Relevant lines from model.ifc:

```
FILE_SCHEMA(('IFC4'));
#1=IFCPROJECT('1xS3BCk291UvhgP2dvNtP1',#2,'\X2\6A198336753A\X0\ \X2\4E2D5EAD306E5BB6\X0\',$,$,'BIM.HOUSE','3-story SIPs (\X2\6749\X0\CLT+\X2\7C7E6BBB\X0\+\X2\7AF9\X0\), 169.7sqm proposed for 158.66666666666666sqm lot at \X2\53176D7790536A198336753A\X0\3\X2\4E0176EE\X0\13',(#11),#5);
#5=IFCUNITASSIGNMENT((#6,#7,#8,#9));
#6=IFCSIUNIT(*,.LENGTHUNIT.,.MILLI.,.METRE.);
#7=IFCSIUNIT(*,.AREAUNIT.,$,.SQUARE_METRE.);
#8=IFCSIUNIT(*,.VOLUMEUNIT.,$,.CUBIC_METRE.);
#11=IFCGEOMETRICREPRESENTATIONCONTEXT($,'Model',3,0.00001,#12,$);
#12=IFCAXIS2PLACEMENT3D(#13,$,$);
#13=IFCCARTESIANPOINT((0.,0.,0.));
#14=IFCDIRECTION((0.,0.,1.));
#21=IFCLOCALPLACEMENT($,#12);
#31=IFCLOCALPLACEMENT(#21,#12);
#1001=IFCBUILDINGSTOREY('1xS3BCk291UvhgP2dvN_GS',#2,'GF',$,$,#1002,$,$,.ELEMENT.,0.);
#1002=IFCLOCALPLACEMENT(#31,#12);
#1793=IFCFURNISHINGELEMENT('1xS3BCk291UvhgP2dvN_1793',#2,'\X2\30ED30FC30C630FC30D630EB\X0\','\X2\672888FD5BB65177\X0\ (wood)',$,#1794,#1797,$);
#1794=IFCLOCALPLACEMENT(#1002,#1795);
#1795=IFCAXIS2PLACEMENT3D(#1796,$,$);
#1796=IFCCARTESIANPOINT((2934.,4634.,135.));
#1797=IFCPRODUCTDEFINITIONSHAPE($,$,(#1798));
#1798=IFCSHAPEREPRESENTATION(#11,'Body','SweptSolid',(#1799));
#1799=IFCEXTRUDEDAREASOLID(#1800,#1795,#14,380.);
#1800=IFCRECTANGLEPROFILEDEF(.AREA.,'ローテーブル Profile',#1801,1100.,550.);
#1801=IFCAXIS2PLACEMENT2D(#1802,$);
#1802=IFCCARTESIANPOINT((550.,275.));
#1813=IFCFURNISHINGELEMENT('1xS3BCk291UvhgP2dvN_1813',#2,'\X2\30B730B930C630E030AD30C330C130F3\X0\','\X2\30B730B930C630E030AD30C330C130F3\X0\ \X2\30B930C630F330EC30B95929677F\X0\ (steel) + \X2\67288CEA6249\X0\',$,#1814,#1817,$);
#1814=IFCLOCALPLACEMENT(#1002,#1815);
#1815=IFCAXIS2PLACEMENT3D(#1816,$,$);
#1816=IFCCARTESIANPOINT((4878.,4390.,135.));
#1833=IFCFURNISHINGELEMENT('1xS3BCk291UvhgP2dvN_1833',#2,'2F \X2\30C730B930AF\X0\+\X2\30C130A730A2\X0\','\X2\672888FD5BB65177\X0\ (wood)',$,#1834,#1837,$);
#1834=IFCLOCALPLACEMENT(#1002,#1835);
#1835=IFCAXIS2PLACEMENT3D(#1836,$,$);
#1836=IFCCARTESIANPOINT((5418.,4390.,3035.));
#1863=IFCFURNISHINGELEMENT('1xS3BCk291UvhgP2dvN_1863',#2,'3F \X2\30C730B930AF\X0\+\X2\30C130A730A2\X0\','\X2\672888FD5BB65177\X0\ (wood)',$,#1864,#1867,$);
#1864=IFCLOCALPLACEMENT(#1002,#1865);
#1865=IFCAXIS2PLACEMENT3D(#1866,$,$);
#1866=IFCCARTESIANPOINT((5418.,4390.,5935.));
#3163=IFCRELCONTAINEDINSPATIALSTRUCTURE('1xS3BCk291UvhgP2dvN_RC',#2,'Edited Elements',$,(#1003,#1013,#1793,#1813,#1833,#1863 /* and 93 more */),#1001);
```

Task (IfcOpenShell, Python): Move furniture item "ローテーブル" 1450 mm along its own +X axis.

```python
import ifcopenshell
import ifcopenshell.api.geometry
import ifcopenshell.util.placement

model = ifcopenshell.open("model.ifc")

item = model.by_guid("1xS3BCk291UvhgP2dvN_1793")
matrix = ifcopenshell.util.placement.get_local_placement(item.ObjectPlacement)
matrix[:3, 3] += matrix[:3, 0] * 1450.0
ifcopenshell.api.geometry.edit_object_placement(model, product=item, matrix=matrix, is_si=False)

print(ifcopenshell.util.placement.get_local_placement(item.ObjectPlacement).round(3) + 0.0)

model.write("model_updated.ifc")
```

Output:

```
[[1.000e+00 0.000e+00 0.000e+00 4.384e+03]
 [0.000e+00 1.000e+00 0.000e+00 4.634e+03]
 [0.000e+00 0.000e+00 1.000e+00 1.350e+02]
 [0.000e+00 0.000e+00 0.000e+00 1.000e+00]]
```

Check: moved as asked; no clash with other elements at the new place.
